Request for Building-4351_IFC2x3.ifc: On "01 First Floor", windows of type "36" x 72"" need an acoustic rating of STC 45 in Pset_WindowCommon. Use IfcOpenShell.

First a look at what the model holds.

```python
import ifcopenshell
import ifcopenshell.util.element

model = ifcopenshell.open("Building-4351_IFC2x3.ifc")
print(model.schema)
storey = next(s for s in model.by_type("IfcBuildingStorey") if s.Name == "01 First Floor")
windows = [e for e in ifcopenshell.util.element.get_decomposition(storey) if e.is_a("IfcWindow")]
seen = {}
for e in windows:
    element_type = ifcopenshell.util.element.get_type(e)
    key = (element_type.Name if element_type != e and element_type else None, ifcopenshell.util.element.get_pset(e, "Pset_WindowCommon", "AcousticRating"))
    seen[key] = seen.get(key, 0) + 1
for (name, value), count in sorted(seen.items(), key=str):
    print(count, "x", name, "|", value)
```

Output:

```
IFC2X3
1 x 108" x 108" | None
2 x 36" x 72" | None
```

```python
import ifcopenshell
import ifcopenshell.api.pset
import ifcopenshell.util.element

model = ifcopenshell.open("Building-4351_IFC2x3.ifc")

storey = next(s for s in model.by_type("IfcBuildingStorey") if s.Name == "01 First Floor")
windows = [e for e in ifcopenshell.util.element.get_decomposition(storey) if e.is_a("IfcWindow")]

count = 0
for e in windows:
    element_type = ifcopenshell.util.element.get_type(e)
    if element_type in (None, e) or element_type.Name != '36" x 72"':
        continue
    # add_pset returns the element's existing set when there is one.
    pset = ifcopenshell.api.pset.add_pset(model, product=e, name="Pset_WindowCommon")
    ifcopenshell.api.pset.edit_pset(model, pset=pset, properties={"AcousticRating": "STC 45"})
    count += 1

print(count, "windows updated")

model.write("Building-4351_IFC2x3-out.ifc")
```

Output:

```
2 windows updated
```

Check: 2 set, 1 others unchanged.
